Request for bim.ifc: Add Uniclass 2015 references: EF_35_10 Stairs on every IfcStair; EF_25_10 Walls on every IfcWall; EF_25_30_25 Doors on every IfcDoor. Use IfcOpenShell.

First a look at what the model holds.

```python
import ifcopenshell

model = ifcopenshell.open("bim.ifc")
print(model.schema)
print("classifications:", [c.Name for c in model.by_type("IfcClassification")])
for ifc_class in ("IfcDoor", "IfcRoof", "IfcStair", "IfcWall", "IfcWindow"):
    print(ifc_class, len(model.by_type(ifc_class)))
```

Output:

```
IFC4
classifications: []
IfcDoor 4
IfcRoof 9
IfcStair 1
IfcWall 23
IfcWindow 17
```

```python
import ifcopenshell
import ifcopenshell.api.classification

model = ifcopenshell.open("bim.ifc")

system = ifcopenshell.api.classification.add_classification(model, classification="Uniclass 2015")

codes = {
    "IfcStair": ("EF_35_10", "Stairs"),
    "IfcWall": ("EF_25_10", "Walls"),
    "IfcDoor": ("EF_25_30_25", "Doors"),
}
for ifc_class, (code, name) in codes.items():
    products = model.by_type(ifc_class)
    ifcopenshell.api.classification.add_reference(
        model, products=products, classification=system, identification=code, name=name
    )
    print(code, len(products))

model.write("bim_updated.ifc")
```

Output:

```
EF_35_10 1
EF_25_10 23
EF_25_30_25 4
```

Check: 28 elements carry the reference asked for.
